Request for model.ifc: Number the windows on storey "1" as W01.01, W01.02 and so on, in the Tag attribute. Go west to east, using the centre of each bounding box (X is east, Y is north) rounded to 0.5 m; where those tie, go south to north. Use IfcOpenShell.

First a look at what the model holds.

```python
import ifcopenshell
import ifcopenshell.util.element
import ifcopenshell.util.placement

model = ifcopenshell.open("model.ifc")
print(model.schema)
storey = next(s for s in model.by_type("IfcBuildingStorey") if s.Name == "1")
windows = [e for e in ifcopenshell.util.element.get_decomposition(storey) if e.is_a("IfcWindow")]
for e in sorted(windows, key=lambda e: e.id()):
    origin = ifcopenshell.util.placement.get_local_placement(e.ObjectPlacement)[:3, 3]
    print(e.id(), e.Tag, e.Name, origin.round(2) + 0.0, sep=" | ")
```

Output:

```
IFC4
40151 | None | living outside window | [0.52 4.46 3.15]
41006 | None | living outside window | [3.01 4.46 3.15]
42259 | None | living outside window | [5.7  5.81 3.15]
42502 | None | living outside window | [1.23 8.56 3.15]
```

```python
import ifcopenshell
import ifcopenshell.geom
import ifcopenshell.util.element
import ifcopenshell.util.shape

model = ifcopenshell.open("model.ifc")
settings = ifcopenshell.geom.settings()
settings.set("use-world-coords", True)


def centre(element):
    shape = ifcopenshell.geom.create_shape(settings, element)
    return ifcopenshell.util.shape.get_bbox_centroid(shape.geometry)


storey = next(s for s in model.by_type("IfcBuildingStorey") if s.Name == "1")
windows = [e for e in ifcopenshell.util.element.get_decomposition(storey) if e.is_a("IfcWindow")]

# Insertion points can sit at a corner or the storey origin, so sort by the geometry (in metres).
centres = {e: centre(e) for e in windows}
windows.sort(key=lambda e: (round(centres[e][0] / 0.5), centres[e][1]))

for i, e in enumerate(windows, start=1):
    number = f"W01.{i:02d}"
    e.Tag = number
    print(e.id(), number)

model.write("model_updated.ifc")
```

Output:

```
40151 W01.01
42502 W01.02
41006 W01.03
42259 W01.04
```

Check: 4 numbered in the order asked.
